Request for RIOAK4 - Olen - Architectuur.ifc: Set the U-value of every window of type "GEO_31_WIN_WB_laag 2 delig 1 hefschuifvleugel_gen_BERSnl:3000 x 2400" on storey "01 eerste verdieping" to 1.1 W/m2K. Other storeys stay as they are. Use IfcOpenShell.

First a look at what the model holds.

```python
import ifcopenshell
import ifcopenshell.util.element

model = ifcopenshell.open("RIOAK4 - Olen - Architectuur.ifc")
print(model.schema)
storey = next(s for s in model.by_type("IfcBuildingStorey") if s.Name == "01 eerste verdieping")
windows = [e for e in ifcopenshell.util.element.get_decomposition(storey) if e.is_a("IfcWindow")]
seen = {}
for e in windows:
    element_type = ifcopenshell.util.element.get_type(e)
    key = (element_type.Name if element_type != e and element_type else None, ifcopenshell.util.element.get_pset(e, "Pset_WindowCommon", "ThermalTransmittance"))
    seen[key] = seen.get(key, 0) + 1
for (name, value), count in sorted(seen.items(), key=str):
    print(count, "x", name, "|", value)
```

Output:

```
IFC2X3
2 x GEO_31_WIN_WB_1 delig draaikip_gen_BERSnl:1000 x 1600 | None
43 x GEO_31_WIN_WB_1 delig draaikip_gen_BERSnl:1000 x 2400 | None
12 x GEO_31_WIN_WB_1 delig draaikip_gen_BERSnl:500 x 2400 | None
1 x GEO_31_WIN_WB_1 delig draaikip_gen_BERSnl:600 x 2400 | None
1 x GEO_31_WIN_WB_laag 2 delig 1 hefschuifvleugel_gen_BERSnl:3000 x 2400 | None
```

```python
import ifcopenshell
import ifcopenshell.api.pset
import ifcopenshell.util.element

model = ifcopenshell.open("RIOAK4 - Olen - Architectuur.ifc")

storey = next(s for s in model.by_type("IfcBuildingStorey") if s.Name == "01 eerste verdieping")
windows = [e for e in ifcopenshell.util.element.get_decomposition(storey) if e.is_a("IfcWindow")]

count = 0
for e in windows:
    element_type = ifcopenshell.util.element.get_type(e)
    if element_type in (None, e) or element_type.Name != "GEO_31_WIN_WB_laag 2 delig 1 hefschuifvleugel_gen_BERSnl:3000 x 2400":
        continue
    # add_pset returns the element's existing set when there is one.
    pset = ifcopenshell.api.pset.add_pset(model, product=e, name="Pset_WindowCommon")
    ifcopenshell.api.pset.edit_pset(model, pset=pset, properties={"ThermalTransmittance": 1.1})
    count += 1

print(count, "windows updated")

model.write("RIOAK4 - Olen - Architectuur_v2.ifc")
```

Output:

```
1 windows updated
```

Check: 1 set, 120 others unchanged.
